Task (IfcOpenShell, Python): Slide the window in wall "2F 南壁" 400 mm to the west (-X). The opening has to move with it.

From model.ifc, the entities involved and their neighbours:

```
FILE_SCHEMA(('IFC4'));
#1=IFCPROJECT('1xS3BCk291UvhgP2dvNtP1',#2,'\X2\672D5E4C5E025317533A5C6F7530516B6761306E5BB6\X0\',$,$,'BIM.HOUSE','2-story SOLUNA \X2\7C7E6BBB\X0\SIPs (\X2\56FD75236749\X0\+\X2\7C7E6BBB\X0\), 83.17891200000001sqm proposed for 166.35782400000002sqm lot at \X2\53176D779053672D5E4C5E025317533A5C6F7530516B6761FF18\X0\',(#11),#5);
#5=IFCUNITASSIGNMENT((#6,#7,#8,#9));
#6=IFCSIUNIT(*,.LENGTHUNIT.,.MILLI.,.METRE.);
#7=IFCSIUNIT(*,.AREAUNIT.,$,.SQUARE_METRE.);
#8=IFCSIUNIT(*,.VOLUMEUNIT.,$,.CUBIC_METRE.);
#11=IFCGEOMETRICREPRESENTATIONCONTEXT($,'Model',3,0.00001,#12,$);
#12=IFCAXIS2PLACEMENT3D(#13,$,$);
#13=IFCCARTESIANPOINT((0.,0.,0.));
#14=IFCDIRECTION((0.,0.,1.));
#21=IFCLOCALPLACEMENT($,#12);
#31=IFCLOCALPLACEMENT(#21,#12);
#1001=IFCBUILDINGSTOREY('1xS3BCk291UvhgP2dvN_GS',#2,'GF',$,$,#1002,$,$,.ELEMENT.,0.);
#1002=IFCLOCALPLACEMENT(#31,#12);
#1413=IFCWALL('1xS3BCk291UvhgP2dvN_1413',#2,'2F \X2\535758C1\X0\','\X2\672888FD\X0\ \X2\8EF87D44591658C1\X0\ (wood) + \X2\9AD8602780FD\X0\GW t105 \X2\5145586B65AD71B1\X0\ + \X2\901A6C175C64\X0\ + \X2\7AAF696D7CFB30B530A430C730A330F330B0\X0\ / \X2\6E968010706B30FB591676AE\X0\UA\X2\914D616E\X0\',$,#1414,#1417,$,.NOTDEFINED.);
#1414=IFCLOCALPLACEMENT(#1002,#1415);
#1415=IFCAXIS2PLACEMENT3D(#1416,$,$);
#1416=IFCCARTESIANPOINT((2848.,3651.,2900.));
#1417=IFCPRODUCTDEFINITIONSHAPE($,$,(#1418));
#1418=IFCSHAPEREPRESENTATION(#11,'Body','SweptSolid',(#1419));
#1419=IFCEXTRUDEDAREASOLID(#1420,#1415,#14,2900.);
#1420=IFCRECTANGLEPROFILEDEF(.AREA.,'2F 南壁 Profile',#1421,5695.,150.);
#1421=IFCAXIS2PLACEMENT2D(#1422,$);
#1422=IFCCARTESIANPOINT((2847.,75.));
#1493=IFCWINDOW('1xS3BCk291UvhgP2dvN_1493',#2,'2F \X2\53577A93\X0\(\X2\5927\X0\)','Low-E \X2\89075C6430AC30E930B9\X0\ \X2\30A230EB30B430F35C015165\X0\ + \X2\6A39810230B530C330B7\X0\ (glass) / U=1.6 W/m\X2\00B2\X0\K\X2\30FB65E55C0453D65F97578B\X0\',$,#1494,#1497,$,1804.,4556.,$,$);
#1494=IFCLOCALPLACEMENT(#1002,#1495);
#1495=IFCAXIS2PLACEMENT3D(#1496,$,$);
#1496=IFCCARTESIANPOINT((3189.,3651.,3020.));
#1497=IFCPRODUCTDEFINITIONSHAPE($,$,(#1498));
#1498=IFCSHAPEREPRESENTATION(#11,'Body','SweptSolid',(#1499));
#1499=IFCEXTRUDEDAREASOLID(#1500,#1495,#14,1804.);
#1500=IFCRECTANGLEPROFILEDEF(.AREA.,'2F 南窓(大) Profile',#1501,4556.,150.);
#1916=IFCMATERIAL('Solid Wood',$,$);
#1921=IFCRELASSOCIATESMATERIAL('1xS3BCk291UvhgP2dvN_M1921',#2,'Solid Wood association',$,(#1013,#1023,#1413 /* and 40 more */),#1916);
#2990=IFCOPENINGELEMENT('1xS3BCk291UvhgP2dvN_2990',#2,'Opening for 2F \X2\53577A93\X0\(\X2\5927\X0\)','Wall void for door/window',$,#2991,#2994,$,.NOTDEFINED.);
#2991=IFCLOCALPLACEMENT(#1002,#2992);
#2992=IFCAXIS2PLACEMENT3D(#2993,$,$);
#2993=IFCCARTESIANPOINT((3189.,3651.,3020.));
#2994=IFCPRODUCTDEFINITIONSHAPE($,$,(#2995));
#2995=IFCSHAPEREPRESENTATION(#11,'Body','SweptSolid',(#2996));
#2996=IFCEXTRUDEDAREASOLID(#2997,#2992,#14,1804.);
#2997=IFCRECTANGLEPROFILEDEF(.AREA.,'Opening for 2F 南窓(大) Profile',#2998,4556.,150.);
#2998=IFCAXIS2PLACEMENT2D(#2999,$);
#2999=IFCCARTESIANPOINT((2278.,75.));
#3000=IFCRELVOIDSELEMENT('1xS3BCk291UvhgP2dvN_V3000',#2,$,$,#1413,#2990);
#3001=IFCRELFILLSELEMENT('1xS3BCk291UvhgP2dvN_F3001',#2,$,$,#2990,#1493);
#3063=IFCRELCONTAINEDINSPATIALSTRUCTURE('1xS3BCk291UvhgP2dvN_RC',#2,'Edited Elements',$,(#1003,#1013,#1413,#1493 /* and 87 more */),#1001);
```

```python
import ifcopenshell
import ifcopenshell.api.geometry
import ifcopenshell.util.placement
import ifcopenshell.util.unit

model = ifcopenshell.open("model.ifc")
unit_scale = ifcopenshell.util.unit.calculate_unit_scale(model)

window = model.by_guid("1xS3BCk291UvhgP2dvN_1493")
opening = window.FillsVoids[0].RelatingOpeningElement
wall = opening.VoidsElements[0].RelatingBuildingElement

wall_matrix = ifcopenshell.util.placement.get_local_placement(wall.ObjectPlacement)
shift = wall_matrix[:3, 0] * -0.4 / unit_scale
before = ifcopenshell.util.placement.get_local_placement(window.ObjectPlacement)[:3, 3].copy()

# The window is not placed relative to its opening, so move both.
for product in (opening, window):
    matrix = ifcopenshell.util.placement.get_local_placement(product.ObjectPlacement)
    matrix[:3, 3] += shift
    ifcopenshell.api.geometry.edit_object_placement(model, product=product, matrix=matrix, is_si=False)

after = ifcopenshell.util.placement.get_local_placement(window.ObjectPlacement)[:3, 3]
print("window moved by", (after - before).round(3) + 0.0)

model.write("model-out.ifc")
```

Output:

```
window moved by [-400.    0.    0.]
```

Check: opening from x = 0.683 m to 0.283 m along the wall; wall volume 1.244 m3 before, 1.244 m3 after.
